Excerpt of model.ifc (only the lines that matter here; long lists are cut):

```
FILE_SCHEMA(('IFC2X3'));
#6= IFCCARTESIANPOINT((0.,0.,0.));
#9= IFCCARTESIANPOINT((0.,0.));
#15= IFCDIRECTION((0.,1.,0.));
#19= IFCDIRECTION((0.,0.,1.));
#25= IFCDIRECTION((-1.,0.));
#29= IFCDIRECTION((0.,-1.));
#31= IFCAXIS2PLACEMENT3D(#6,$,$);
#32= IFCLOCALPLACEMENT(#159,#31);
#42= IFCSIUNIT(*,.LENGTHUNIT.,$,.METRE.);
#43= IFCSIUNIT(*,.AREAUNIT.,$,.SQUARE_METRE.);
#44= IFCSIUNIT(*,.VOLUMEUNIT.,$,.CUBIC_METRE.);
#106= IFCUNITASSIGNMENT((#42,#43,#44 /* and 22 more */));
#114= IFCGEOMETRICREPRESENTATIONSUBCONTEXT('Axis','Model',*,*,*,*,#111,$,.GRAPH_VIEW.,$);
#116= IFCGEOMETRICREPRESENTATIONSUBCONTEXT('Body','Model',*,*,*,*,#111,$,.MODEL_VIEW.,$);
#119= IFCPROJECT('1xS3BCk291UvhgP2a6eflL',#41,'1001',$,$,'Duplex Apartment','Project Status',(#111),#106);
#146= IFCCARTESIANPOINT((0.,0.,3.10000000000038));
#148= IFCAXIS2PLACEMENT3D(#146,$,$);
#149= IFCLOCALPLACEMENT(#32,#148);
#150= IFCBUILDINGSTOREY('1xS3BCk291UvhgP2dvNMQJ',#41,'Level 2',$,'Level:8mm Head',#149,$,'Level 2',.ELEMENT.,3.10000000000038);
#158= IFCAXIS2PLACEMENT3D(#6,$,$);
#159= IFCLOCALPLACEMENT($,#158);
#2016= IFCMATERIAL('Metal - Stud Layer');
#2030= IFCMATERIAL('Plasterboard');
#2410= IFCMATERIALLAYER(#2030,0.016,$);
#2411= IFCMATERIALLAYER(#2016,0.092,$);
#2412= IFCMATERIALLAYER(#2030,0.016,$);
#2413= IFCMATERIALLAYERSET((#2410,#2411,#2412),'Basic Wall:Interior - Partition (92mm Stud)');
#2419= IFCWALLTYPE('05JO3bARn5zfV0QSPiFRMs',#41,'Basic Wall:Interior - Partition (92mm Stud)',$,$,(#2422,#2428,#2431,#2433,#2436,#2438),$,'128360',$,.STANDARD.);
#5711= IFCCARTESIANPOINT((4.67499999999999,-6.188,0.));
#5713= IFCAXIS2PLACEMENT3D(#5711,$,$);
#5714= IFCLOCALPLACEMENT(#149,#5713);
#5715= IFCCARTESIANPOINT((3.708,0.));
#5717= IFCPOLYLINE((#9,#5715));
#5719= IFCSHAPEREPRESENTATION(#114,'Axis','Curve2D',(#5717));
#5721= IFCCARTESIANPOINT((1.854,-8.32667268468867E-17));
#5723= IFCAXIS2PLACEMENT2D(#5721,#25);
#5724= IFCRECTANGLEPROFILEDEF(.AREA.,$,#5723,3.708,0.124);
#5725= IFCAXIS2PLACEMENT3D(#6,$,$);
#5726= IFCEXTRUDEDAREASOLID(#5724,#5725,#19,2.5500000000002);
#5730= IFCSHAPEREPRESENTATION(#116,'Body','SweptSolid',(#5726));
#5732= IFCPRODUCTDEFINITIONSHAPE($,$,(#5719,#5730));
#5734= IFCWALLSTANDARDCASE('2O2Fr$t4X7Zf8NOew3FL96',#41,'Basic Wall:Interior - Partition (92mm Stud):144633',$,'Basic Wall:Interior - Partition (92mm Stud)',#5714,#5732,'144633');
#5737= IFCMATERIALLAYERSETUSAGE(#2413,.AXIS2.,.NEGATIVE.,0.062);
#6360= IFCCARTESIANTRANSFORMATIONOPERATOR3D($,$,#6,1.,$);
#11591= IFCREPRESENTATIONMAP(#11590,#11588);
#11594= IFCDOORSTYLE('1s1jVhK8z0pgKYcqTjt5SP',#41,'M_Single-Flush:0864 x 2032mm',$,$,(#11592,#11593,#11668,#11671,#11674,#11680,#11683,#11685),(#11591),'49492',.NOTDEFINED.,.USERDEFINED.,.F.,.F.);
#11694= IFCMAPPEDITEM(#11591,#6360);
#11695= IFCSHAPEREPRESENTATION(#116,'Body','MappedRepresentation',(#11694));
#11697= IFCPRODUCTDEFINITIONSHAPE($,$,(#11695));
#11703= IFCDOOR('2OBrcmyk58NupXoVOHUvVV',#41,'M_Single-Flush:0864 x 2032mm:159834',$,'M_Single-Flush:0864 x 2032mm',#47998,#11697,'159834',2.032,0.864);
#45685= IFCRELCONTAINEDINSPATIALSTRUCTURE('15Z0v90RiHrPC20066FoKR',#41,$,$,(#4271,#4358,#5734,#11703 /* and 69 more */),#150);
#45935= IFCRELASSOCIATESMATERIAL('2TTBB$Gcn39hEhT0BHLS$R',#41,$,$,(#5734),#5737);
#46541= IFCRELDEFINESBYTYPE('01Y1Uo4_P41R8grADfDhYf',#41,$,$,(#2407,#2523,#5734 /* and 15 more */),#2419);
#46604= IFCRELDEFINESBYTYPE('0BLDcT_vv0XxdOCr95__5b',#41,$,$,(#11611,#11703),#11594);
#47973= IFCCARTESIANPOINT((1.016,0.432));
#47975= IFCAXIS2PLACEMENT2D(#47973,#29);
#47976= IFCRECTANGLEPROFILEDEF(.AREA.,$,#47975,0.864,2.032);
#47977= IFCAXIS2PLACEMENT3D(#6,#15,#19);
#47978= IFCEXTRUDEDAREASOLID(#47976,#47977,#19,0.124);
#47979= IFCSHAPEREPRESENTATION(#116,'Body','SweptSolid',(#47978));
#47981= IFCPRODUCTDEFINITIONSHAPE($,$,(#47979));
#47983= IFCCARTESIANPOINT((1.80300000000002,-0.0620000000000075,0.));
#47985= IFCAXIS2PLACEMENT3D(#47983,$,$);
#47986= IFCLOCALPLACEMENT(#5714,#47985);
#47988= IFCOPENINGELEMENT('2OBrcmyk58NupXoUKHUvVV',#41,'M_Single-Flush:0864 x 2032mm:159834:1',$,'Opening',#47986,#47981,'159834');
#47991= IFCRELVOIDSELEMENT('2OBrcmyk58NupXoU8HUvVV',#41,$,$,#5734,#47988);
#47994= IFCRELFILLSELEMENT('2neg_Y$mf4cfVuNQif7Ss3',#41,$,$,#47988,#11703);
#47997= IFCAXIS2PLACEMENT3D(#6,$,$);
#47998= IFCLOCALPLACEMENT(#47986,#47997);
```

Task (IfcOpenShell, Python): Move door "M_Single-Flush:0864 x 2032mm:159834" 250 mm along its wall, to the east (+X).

```python
import ifcopenshell
import ifcopenshell.api.geometry
import ifcopenshell.util.placement

model = ifcopenshell.open("model.ifc")

door = model.by_guid("2OBrcmyk58NupXoVOHUvVV")
opening = door.FillsVoids[0].RelatingOpeningElement
wall = opening.VoidsElements[0].RelatingBuildingElement

wall_matrix = ifcopenshell.util.placement.get_local_placement(wall.ObjectPlacement)
shift = wall_matrix[:3, 0] * 0.25
before = ifcopenshell.util.placement.get_local_placement(door.ObjectPlacement)[:3, 3].copy()

# The door is placed relative to its opening, so it follows when the opening moves.
matrix = ifcopenshell.util.placement.get_local_placement(opening.ObjectPlacement)
matrix[:3, 3] += shift
ifcopenshell.api.geometry.edit_object_placement(
    model, product=opening, matrix=matrix, is_si=False, should_transform_children=True
)

after = ifcopenshell.util.placement.get_local_placement(door.ObjectPlacement)[:3, 3]
print("door moved by", (after - before).round(3) + 0.0)

model.write("model_updated.ifc")
```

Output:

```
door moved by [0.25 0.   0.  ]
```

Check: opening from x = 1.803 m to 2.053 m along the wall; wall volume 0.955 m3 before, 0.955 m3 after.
